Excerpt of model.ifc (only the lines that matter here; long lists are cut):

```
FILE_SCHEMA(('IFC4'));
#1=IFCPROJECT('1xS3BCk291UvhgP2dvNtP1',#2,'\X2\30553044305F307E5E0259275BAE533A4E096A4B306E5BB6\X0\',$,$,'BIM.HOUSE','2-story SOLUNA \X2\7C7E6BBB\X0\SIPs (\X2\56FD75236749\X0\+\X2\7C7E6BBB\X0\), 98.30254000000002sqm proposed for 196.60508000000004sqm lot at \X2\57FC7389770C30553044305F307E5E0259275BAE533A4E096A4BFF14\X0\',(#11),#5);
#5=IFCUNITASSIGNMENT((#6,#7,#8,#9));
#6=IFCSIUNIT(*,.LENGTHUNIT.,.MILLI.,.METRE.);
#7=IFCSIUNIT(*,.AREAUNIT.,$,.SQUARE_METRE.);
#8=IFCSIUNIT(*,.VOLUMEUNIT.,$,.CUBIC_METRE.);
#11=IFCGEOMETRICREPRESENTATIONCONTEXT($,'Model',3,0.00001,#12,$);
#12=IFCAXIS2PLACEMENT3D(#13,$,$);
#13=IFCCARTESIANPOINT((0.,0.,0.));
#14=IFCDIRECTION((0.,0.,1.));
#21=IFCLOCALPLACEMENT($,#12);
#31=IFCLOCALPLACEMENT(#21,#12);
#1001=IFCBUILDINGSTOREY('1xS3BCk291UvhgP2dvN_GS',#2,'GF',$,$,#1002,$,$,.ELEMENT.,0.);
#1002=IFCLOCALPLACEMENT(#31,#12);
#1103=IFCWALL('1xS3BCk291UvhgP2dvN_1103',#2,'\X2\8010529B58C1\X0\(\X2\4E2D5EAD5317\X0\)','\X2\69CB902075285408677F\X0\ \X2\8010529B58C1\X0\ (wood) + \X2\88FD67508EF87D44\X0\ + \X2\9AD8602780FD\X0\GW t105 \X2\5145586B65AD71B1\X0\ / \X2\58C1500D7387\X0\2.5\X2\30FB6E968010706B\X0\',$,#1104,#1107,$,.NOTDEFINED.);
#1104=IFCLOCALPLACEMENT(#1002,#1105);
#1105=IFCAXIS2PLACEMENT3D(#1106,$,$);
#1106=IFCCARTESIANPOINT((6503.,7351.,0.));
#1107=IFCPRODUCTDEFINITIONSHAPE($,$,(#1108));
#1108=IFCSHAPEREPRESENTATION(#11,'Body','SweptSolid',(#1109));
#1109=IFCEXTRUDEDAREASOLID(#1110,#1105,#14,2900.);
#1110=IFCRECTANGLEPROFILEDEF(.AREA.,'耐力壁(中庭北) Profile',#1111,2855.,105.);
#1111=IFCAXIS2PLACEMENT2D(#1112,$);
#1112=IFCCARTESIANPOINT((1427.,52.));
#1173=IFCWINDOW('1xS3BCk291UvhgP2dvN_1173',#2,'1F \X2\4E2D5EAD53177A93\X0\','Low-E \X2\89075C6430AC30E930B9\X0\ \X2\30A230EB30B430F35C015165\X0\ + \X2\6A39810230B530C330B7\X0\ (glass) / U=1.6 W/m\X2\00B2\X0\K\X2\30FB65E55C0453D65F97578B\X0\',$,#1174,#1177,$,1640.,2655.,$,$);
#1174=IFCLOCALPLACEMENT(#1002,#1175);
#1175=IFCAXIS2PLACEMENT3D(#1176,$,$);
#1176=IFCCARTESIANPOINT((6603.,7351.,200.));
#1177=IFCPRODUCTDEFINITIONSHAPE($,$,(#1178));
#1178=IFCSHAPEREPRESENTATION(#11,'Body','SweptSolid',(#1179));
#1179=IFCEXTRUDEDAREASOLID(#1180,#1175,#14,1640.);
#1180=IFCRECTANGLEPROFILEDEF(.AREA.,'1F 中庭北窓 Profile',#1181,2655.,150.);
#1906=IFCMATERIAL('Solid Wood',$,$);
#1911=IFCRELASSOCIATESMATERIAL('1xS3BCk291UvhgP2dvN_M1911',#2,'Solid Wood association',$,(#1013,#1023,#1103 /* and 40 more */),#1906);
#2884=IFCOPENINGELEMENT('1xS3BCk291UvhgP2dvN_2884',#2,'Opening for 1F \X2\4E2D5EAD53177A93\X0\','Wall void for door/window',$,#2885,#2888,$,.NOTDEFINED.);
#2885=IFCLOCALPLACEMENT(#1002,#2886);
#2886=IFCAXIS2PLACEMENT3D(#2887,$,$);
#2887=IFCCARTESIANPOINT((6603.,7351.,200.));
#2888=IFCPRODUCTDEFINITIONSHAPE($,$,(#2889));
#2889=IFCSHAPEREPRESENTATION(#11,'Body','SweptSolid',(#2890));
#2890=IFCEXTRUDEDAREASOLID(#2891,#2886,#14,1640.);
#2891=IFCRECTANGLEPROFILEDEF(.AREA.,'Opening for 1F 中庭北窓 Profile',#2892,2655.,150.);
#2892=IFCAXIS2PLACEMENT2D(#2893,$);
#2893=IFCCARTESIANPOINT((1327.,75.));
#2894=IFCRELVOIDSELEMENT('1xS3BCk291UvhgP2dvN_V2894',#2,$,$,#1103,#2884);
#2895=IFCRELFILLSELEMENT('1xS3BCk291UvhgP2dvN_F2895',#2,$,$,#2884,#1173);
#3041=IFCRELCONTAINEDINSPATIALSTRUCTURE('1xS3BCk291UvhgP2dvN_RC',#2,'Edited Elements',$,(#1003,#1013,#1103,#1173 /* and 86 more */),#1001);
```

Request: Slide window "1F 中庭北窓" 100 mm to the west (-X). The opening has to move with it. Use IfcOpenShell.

```python
import ifcopenshell
import ifcopenshell.api.geometry
import ifcopenshell.util.placement
import ifcopenshell.util.unit

model = ifcopenshell.open("model.ifc")
unit_scale = ifcopenshell.util.unit.calculate_unit_scale(model)

window = model.by_guid("1xS3BCk291UvhgP2dvN_1173")
opening = window.FillsVoids[0].RelatingOpeningElement
wall = opening.VoidsElements[0].RelatingBuildingElement

wall_matrix = ifcopenshell.util.placement.get_local_placement(wall.ObjectPlacement)
shift = wall_matrix[:3, 0] * -0.1 / unit_scale
before = ifcopenshell.util.placement.get_local_placement(window.ObjectPlacement)[:3, 3].copy()

# The window is not placed relative to its opening, so move both.
for product in (opening, window):
    matrix = ifcopenshell.util.placement.get_local_placement(product.ObjectPlacement)
    matrix[:3, 3] += shift
    ifcopenshell.api.geometry.edit_object_placement(model, product=product, matrix=matrix, is_si=False)

after = ifcopenshell.util.placement.get_local_placement(window.ObjectPlacement)[:3, 3]
print("window moved by", (after - before).round(3) + 0.0)

model.write("model_v2.ifc")
```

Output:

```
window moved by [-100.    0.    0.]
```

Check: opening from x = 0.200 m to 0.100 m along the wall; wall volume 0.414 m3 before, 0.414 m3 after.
